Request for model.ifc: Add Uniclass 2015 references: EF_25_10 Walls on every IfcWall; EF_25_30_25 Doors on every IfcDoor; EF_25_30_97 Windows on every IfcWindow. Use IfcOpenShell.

First a look at what the model holds.

```python
import ifcopenshell

model = ifcopenshell.open("model.ifc")
print(model.schema)
print("classifications:", [c.Name for c in model.by_type("IfcClassification")])
for ifc_class in ("IfcDoor", "IfcRoof", "IfcStair", "IfcWall", "IfcWindow"):
    print(ifc_class, len(model.by_type(ifc_class)))
```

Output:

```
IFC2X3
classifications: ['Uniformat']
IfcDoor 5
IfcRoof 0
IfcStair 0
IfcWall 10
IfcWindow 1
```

```python
import ifcopenshell
import ifcopenshell.api.classification

model = ifcopenshell.open("model.ifc")

# IFC2X3 requires Source and Edition and has no link from the project to the system.
system = model.create_entity("IfcClassification", Source="NBS", Edition="2015", Name="Uniclass 2015")

codes = {
    "IfcWall": ("EF_25_10", "Walls"),
    "IfcDoor": ("EF_25_30_25", "Doors"),
    "IfcWindow": ("EF_25_30_97", "Windows"),
}
for ifc_class, (code, name) in codes.items():
    products = model.by_type(ifc_class)
    ifcopenshell.api.classification.add_reference(
        model, products=products, classification=system, identification=code, name=name
    )
    print(code, len(products))

model.write("model_edited.ifc")
```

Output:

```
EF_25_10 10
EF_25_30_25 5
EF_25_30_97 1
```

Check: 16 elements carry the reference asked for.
